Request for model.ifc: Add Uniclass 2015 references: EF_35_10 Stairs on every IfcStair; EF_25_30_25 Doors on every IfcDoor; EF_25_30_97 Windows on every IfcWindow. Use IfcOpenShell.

First a look at what the model holds.

```python
import ifcopenshell

model = ifcopenshell.open("model.ifc")
print(model.schema)
print("classifications:", [c.Name for c in model.by_type("IfcClassification")])
for ifc_class in ("IfcDoor", "IfcRoof", "IfcStair", "IfcWall", "IfcWindow"):
    print(ifc_class, len(model.by_type(ifc_class)))
```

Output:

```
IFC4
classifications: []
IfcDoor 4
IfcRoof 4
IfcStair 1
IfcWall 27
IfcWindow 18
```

```python
import ifcopenshell
import ifcopenshell.api.classification

model = ifcopenshell.open("model.ifc")

system = ifcopenshell.api.classification.add_classification(model, classification="Uniclass 2015")

codes = {
    "IfcStair": ("EF_35_10", "Stairs"),
    "IfcDoor": ("EF_25_30_25", "Doors"),
    "IfcWindow": ("EF_25_30_97", "Windows"),
}
for ifc_class, (code, name) in codes.items():
    products = model.by_type(ifc_class)
    ifcopenshell.api.classification.add_reference(
        model, products=products, classification=system, identification=code, name=name
    )
    print(code, len(products))

model.write("model_rev.ifc")
```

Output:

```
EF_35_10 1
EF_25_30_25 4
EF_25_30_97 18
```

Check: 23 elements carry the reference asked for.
